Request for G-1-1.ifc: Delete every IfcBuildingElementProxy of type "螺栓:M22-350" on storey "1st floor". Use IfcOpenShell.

First a look at what the model holds.

```python
import ifcopenshell
import ifcopenshell.util.element

model = ifcopenshell.open("G-1-1.ifc")
print(model.schema)
storey = next(s for s in model.by_type("IfcBuildingStorey") if s.Name == "1st floor")
proxies = [e for e in ifcopenshell.util.element.get_decomposition(storey) if e.is_a("IfcBuildingElementProxy")]
seen = {}
for e in proxies:
    element_type = ifcopenshell.util.element.get_type(e)
    name = element_type.Name if element_type not in (None, e) else None
    seen[name] = seen.get(name, 0) + 1
for name, count in sorted(seen.items(), key=str):
    print(count, "x", name)
```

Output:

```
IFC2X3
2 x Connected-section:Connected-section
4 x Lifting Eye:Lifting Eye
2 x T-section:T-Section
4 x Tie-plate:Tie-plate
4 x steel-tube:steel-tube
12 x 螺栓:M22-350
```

```python
import ifcopenshell
import ifcopenshell.api.root
import ifcopenshell.util.element

model = ifcopenshell.open("G-1-1.ifc")

storey = next(s for s in model.by_type("IfcBuildingStorey") if s.Name == "1st floor")
proxies = [e for e in ifcopenshell.util.element.get_decomposition(storey) if e.is_a("IfcBuildingElementProxy")]
targets = [e for e in proxies if (t := ifcopenshell.util.element.get_type(e)) not in (None, e) and t.Name == "螺栓:M22-350"]

for e in targets:
    ifcopenshell.api.root.remove_product(model, product=e)
print(len(targets), "removed")

model.write("G-1-1_v2.ifc")
```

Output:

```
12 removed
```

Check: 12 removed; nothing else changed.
